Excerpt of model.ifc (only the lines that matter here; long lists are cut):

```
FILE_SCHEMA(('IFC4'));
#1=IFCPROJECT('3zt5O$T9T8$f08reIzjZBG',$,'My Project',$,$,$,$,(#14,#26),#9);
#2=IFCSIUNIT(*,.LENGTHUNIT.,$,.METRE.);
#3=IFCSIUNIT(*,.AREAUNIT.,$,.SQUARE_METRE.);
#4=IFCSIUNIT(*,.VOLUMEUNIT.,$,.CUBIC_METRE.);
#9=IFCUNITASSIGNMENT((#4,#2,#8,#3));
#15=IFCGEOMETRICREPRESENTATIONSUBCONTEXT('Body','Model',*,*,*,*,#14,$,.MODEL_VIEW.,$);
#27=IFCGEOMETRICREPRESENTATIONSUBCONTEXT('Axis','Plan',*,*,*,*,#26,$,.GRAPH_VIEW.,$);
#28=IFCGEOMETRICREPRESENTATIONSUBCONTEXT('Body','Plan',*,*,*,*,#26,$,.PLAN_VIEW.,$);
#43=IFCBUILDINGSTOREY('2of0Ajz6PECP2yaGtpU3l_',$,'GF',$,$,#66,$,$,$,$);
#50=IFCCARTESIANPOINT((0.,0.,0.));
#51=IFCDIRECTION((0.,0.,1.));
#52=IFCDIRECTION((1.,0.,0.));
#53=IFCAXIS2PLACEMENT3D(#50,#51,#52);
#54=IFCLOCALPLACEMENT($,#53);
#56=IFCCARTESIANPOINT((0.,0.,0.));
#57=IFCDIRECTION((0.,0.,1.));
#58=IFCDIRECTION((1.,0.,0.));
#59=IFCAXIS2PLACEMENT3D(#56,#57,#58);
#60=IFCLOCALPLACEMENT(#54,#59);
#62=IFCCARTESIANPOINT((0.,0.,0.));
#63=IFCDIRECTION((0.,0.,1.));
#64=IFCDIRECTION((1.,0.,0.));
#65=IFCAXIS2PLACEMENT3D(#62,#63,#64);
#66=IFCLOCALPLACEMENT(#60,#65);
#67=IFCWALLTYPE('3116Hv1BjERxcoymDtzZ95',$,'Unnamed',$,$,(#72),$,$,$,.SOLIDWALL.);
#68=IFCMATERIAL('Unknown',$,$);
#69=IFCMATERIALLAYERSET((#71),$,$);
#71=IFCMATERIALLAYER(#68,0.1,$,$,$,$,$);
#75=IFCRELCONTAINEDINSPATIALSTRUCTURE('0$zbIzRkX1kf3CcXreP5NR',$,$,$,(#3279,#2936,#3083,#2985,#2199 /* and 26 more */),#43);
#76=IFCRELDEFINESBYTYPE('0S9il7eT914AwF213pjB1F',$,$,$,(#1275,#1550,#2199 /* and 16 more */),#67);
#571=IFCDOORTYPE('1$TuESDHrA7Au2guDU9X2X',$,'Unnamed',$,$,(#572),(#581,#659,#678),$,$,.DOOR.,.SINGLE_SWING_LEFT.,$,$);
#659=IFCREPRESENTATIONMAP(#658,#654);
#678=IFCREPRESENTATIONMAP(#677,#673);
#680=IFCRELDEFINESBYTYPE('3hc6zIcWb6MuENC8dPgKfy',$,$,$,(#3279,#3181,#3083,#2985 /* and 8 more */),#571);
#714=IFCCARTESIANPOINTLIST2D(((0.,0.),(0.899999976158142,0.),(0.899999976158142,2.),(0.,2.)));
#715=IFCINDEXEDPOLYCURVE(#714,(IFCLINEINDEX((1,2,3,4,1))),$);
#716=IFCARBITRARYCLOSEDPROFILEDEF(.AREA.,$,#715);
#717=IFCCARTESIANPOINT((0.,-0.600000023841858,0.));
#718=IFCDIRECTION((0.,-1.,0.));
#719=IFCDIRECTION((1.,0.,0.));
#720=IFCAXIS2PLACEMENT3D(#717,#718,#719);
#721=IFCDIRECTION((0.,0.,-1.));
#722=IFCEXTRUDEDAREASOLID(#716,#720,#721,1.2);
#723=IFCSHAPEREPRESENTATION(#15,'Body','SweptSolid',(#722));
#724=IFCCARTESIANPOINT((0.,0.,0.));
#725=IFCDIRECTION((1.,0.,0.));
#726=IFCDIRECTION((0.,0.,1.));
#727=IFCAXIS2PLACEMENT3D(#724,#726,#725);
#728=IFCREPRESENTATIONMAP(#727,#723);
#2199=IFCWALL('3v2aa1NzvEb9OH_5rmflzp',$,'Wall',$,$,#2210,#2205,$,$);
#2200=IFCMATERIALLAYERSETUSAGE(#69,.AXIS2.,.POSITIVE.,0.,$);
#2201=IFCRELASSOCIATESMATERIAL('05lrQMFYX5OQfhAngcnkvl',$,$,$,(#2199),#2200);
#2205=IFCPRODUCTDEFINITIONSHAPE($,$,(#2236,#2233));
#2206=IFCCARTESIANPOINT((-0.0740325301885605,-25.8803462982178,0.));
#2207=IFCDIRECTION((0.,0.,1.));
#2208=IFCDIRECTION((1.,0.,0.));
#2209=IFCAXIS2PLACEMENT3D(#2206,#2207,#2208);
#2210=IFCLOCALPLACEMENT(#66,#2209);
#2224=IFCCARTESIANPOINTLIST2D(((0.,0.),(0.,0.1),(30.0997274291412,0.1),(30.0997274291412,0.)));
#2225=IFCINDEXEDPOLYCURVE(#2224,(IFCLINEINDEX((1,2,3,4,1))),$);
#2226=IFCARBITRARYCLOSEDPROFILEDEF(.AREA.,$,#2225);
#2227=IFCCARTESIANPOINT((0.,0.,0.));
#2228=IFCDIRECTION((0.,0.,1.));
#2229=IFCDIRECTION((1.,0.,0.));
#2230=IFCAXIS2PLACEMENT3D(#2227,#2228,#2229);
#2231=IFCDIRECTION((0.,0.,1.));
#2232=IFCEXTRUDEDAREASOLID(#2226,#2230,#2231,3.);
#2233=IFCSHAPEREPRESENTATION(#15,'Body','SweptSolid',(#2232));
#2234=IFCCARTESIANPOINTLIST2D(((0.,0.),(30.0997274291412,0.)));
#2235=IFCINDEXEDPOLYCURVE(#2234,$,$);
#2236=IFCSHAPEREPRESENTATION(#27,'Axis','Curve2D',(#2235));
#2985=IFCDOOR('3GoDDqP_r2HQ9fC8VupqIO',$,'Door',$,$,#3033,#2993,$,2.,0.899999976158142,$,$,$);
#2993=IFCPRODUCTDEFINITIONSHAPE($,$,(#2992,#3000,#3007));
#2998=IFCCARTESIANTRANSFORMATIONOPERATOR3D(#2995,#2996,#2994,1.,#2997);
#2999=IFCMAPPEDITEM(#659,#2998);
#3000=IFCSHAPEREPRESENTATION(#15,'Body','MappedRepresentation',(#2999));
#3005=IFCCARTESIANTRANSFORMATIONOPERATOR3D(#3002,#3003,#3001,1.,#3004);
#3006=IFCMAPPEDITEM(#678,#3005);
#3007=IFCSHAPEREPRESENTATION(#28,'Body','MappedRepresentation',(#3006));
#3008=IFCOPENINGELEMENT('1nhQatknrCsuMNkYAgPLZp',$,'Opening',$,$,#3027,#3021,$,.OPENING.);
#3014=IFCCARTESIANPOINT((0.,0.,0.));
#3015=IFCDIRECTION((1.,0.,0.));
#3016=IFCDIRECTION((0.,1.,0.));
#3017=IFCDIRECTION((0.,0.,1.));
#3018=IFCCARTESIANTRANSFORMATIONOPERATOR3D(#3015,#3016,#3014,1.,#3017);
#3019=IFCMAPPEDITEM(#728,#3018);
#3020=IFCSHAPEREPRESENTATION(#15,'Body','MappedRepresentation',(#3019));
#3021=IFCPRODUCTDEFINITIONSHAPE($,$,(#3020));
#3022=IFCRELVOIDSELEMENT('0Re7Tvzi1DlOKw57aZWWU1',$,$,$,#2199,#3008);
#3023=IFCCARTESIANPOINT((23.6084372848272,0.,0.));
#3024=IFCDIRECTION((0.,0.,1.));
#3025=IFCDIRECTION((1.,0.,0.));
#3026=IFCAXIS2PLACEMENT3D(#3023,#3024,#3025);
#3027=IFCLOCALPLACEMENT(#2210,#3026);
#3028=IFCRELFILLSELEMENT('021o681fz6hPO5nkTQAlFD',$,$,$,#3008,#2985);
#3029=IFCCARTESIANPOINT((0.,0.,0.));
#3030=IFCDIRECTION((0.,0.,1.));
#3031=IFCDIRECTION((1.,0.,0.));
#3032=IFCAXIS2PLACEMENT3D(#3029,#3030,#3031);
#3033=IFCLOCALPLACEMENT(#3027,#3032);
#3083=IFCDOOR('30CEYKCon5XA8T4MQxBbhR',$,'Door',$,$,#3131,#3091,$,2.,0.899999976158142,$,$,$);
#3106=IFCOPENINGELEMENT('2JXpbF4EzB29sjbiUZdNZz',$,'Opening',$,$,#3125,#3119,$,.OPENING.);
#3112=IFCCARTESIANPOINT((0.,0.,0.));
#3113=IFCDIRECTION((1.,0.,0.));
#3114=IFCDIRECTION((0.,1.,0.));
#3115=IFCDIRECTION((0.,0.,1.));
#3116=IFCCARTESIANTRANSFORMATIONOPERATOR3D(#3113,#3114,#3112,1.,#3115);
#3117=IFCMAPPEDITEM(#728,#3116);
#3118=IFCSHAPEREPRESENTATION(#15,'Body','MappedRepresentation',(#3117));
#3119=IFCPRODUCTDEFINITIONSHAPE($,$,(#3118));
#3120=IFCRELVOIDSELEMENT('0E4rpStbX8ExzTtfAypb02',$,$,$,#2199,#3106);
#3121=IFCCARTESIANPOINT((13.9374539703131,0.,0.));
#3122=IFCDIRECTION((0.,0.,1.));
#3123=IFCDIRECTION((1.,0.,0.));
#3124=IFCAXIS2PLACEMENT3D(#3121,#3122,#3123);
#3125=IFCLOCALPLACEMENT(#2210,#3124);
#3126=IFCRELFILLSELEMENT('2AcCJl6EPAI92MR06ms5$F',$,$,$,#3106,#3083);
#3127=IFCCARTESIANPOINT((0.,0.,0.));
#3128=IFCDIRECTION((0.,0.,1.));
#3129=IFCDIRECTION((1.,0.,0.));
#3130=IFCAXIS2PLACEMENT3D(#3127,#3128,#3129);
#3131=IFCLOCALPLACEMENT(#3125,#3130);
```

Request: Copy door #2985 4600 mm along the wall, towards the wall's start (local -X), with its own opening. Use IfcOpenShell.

```python
import ifcopenshell
import ifcopenshell.api.feature
import ifcopenshell.api.geometry
import ifcopenshell.api.root
import ifcopenshell.geom
import ifcopenshell.util.element
import ifcopenshell.util.placement
import ifcopenshell.util.shape

model = ifcopenshell.open("model.ifc")
settings = ifcopenshell.geom.settings()


def volume(element):
    """Net volume in cubic metres, openings subtracted."""
    shape = ifcopenshell.geom.create_shape(settings, element)
    return ifcopenshell.util.shape.get_volume(shape.geometry)


door = model.by_id(2985)
opening = door.FillsVoids[0].RelatingOpeningElement
wall = opening.VoidsElements[0].RelatingBuildingElement
before = volume(wall)
shift = ifcopenshell.util.placement.get_local_placement(wall.ObjectPlacement)[:3, 0] * -4.6

# copy_class copies the void relationship, type, container and properties, but no geometry.
new_opening = ifcopenshell.api.root.copy_class(model, product=opening)
new_opening.Representation = ifcopenshell.util.element.copy_deep(
    model, opening.Representation, exclude=["IfcGeometricRepresentationContext", "IfcRepresentationMap"]
)
new_door = ifcopenshell.api.root.copy_class(model, product=door)
new_door.Representation = ifcopenshell.util.element.copy_deep(
    model, door.Representation, exclude=["IfcGeometricRepresentationContext", "IfcRepresentationMap"]
)
ifcopenshell.api.feature.add_filling(model, opening=new_opening, element=new_door)

for old, new in ((opening, new_opening), (door, new_door)):
    matrix = ifcopenshell.util.placement.get_local_placement(old.ObjectPlacement)
    matrix[:3, 3] += shift
    ifcopenshell.api.geometry.edit_object_placement(model, product=new, matrix=matrix, is_si=False)

after = volume(wall)

print(f"wall volume {before:.3f} -> {after:.3f} m3")

model.write("model-out.ifc")
```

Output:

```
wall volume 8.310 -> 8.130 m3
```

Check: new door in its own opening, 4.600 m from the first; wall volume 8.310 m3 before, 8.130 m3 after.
